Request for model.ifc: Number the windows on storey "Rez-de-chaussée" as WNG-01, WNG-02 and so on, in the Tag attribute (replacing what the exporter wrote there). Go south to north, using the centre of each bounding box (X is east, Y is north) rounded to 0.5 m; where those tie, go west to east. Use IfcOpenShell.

First a look at what the model holds.

```python
import ifcopenshell
import ifcopenshell.util.element
import ifcopenshell.util.placement

model = ifcopenshell.open("model.ifc")
print(model.schema)
storey = next(s for s in model.by_type("IfcBuildingStorey") if s.Name == "Rez-de-chaussée")
windows = [e for e in ifcopenshell.util.element.get_decomposition(storey) if e.is_a("IfcWindow")]
for e in sorted(windows, key=lambda e: e.id()):
    origin = ifcopenshell.util.placement.get_local_placement(e.ObjectPlacement)[:3, 3]
    print(e.id(), e.Tag, e.Name, origin.round(2) + 0.0, sep=" | ")
```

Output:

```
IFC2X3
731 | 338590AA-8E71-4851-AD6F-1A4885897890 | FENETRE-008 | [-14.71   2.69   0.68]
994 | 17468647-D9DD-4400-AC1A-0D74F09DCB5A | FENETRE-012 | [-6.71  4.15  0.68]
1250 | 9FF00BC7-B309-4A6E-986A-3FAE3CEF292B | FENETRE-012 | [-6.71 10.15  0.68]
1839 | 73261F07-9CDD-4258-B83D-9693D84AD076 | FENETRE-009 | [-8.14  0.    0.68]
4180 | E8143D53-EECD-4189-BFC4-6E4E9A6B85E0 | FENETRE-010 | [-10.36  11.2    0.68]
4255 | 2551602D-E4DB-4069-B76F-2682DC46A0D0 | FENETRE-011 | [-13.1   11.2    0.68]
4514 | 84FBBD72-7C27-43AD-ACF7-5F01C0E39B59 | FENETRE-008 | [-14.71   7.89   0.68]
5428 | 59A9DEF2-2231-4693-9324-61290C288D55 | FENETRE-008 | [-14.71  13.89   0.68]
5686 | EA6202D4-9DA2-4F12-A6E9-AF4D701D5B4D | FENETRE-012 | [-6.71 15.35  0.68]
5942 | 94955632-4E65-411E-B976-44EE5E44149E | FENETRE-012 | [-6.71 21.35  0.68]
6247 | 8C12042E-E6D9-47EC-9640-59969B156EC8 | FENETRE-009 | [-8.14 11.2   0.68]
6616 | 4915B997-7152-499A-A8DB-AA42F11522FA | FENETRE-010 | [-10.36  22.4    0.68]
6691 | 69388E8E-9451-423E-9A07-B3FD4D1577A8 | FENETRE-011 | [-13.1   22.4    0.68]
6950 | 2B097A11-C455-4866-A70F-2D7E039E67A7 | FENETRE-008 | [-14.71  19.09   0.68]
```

```python
import ifcopenshell
import ifcopenshell.geom
import ifcopenshell.util.element
import ifcopenshell.util.shape

model = ifcopenshell.open("model.ifc")
settings = ifcopenshell.geom.settings()
settings.set("use-world-coords", True)


def centre(element):
    shape = ifcopenshell.geom.create_shape(settings, element)
    return ifcopenshell.util.shape.get_bbox_centroid(shape.geometry)


storey = next(s for s in model.by_type("IfcBuildingStorey") if s.Name == "Rez-de-chaussée")
windows = [e for e in ifcopenshell.util.element.get_decomposition(storey) if e.is_a("IfcWindow")]

# Insertion points can sit at a corner or the storey origin, so sort by the geometry (in metres).
centres = {e: centre(e) for e in windows}
windows.sort(key=lambda e: (round(centres[e][1] / 0.5), centres[e][0]))

for i, e in enumerate(windows, start=1):
    number = f"WNG-{i:02d}"
    e.Tag = number
    print(e.id(), number)

model.write("model_updated.ifc")
```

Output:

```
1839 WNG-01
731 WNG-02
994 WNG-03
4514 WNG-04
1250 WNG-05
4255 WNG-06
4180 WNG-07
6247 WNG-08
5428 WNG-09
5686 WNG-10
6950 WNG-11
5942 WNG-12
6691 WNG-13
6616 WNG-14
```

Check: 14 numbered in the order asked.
